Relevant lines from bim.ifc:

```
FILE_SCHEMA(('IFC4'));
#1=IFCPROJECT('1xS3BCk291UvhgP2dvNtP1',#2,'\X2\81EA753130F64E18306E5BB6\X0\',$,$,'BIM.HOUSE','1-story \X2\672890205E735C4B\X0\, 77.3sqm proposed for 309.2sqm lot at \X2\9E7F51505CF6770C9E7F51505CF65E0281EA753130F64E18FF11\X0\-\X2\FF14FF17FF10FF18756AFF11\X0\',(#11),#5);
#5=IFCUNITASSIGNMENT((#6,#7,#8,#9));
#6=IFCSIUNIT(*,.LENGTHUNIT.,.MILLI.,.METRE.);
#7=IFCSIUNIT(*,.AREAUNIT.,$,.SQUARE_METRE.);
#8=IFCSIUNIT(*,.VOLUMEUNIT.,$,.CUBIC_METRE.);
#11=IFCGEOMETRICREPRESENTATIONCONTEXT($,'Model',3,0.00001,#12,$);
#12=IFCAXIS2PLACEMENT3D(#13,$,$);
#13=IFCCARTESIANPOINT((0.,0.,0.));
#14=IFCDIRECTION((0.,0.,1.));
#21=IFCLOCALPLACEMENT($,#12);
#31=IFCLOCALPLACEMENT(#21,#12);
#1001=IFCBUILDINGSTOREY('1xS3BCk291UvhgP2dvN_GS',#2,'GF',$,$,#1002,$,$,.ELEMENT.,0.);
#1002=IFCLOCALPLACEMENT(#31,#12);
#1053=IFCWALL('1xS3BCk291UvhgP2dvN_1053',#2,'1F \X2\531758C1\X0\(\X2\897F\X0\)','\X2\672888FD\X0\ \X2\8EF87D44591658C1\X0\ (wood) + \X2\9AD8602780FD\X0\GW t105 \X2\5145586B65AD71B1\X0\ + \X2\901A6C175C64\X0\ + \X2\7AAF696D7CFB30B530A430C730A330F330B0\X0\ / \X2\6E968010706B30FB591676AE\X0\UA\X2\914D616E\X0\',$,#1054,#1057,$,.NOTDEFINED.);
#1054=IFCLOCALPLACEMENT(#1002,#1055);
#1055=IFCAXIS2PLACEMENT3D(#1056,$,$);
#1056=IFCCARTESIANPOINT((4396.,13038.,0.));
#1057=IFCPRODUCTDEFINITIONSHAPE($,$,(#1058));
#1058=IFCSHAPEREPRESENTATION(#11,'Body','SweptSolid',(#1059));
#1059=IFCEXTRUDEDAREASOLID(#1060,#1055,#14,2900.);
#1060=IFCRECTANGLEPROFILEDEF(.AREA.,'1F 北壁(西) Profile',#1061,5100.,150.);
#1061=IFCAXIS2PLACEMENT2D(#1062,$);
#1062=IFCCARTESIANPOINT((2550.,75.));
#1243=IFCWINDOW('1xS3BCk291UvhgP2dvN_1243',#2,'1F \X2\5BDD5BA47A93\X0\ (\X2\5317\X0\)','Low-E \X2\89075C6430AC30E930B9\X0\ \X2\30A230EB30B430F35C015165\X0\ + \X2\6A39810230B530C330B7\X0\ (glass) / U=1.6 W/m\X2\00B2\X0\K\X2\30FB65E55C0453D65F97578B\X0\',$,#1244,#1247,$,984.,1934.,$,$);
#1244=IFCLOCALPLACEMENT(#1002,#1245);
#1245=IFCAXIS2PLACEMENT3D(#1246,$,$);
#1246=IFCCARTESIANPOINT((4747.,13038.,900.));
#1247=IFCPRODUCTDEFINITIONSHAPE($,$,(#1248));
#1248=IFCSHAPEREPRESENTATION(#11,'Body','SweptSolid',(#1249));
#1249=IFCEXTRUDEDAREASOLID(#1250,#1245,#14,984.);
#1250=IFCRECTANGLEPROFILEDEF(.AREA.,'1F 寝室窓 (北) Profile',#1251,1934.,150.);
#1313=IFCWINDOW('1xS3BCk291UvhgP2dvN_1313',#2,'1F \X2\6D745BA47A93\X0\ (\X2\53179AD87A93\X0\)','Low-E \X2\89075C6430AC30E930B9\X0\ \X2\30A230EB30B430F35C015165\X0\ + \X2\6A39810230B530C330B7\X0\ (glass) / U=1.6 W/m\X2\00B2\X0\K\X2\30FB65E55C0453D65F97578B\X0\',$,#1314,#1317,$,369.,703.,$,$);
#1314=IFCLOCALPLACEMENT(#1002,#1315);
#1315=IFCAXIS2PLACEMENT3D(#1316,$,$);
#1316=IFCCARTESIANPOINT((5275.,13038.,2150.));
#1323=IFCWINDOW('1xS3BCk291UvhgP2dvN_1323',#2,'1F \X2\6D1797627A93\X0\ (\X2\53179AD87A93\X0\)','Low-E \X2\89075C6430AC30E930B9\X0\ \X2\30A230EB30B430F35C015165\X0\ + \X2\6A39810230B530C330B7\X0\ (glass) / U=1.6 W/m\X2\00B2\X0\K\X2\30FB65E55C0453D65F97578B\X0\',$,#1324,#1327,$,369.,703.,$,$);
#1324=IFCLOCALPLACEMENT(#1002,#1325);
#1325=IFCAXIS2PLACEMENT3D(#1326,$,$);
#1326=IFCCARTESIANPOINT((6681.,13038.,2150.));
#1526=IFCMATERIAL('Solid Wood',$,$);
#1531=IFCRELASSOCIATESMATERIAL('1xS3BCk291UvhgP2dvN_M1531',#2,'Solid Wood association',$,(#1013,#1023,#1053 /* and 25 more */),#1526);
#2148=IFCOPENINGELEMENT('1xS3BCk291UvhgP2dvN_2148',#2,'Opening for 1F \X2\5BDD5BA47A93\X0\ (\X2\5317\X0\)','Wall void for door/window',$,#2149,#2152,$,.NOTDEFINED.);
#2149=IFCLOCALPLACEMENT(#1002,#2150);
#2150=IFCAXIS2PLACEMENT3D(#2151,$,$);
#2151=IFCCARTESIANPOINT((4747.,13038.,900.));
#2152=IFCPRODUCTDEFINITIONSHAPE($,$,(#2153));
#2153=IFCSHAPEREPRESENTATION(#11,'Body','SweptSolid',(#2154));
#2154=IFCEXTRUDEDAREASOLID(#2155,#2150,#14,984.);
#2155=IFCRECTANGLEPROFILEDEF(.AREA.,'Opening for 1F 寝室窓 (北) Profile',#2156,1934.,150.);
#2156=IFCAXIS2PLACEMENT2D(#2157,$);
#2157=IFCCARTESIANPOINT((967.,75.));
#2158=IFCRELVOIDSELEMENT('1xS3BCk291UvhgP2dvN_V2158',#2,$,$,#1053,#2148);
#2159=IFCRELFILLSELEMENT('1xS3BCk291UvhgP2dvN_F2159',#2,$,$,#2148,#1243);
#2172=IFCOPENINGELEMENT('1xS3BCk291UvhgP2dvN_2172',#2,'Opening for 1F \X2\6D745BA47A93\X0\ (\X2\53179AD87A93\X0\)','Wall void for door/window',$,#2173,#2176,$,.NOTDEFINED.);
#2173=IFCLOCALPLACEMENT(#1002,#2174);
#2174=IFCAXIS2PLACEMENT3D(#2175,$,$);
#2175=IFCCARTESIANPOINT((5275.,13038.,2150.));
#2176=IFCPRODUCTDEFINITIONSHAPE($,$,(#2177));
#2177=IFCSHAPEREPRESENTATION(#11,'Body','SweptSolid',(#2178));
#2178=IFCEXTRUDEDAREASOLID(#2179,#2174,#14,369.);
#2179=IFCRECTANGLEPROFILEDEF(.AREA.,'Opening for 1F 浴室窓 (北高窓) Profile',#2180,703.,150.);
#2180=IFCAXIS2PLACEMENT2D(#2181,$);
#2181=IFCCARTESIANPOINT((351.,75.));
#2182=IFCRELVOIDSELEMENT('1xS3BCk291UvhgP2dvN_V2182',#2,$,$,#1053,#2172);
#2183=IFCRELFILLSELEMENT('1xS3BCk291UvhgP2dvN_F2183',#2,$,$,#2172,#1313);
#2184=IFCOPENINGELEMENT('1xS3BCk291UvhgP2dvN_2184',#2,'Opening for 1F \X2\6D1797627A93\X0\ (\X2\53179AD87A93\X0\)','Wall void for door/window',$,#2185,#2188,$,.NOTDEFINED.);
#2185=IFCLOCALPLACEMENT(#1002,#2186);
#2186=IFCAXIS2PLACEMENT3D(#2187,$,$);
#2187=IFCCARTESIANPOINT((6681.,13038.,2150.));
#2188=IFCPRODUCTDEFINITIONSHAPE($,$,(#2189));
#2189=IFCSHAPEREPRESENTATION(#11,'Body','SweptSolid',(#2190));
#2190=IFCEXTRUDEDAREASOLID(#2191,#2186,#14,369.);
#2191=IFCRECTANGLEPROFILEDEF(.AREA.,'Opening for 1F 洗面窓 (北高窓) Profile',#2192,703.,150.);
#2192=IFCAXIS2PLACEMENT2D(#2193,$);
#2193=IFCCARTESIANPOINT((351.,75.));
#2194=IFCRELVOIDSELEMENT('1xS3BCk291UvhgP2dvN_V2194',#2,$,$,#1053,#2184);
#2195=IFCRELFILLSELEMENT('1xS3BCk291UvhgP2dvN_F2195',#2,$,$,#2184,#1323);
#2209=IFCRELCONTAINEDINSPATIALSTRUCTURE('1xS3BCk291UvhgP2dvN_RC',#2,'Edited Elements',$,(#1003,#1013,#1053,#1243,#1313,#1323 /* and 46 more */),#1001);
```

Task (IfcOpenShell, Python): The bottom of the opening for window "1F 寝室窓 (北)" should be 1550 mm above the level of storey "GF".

```python
import numpy as np
import ifcopenshell
import ifcopenshell.api.geometry
import ifcopenshell.geom
import ifcopenshell.util.element
import ifcopenshell.util.placement
import ifcopenshell.util.shape
import ifcopenshell.util.unit

model = ifcopenshell.open("bim.ifc")
unit_scale = ifcopenshell.util.unit.calculate_unit_scale(model)

window = model.by_guid("1xS3BCk291UvhgP2dvN_1243")
opening = window.FillsVoids[0].RelatingOpeningElement
storey = ifcopenshell.util.element.get_container(window, ifc_class="IfcBuildingStorey")
level = ifcopenshell.util.placement.get_local_placement(storey.ObjectPlacement)[2, 3]

# The opening's origin need not be at the sill, so measure its lowest point.
shape = ifcopenshell.geom.create_shape(ifcopenshell.geom.settings(), opening)
bottom = ifcopenshell.util.shape.get_shape_bottom_elevation(shape, shape.geometry) / unit_scale
dz = level + 1550.0 - bottom

shift = np.array([0.0, 0.0, dz])
# The window is not placed relative to its opening, so move both.
for product in (opening, window):
    matrix = ifcopenshell.util.placement.get_local_placement(product.ObjectPlacement)
    matrix[:3, 3] += shift
    ifcopenshell.api.geometry.edit_object_placement(model, product=product, matrix=matrix, is_si=False)

print(f"moved by {dz * unit_scale:+.3f} m")

model.write("bim_v2.ifc")
```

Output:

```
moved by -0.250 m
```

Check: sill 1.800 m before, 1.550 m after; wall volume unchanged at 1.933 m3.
